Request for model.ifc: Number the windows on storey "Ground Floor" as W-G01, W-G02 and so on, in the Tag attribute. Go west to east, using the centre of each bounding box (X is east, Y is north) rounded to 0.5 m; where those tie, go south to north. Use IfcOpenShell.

First a look at what the model holds.

```python
import ifcopenshell
import ifcopenshell.util.element
import ifcopenshell.util.placement

model = ifcopenshell.open("model.ifc")
print(model.schema)
storey = next(s for s in model.by_type("IfcBuildingStorey") if s.Name == "Ground Floor")
windows = [e for e in ifcopenshell.util.element.get_decomposition(storey) if e.is_a("IfcWindow")]
for e in sorted(windows, key=lambda e: e.id()):
    origin = ifcopenshell.util.placement.get_local_placement(e.ObjectPlacement)[:3, 3]
    print(e.id(), e.Tag, e.Name, origin.round(2) + 0.0, sep=" | ")
```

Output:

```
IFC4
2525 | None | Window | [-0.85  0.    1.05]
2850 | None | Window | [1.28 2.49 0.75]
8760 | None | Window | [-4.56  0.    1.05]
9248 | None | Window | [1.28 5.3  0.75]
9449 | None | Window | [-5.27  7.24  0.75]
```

```python
import ifcopenshell
import ifcopenshell.geom
import ifcopenshell.util.element
import ifcopenshell.util.shape

model = ifcopenshell.open("model.ifc")
settings = ifcopenshell.geom.settings()
settings.set("use-world-coords", True)


def centre(element):
    shape = ifcopenshell.geom.create_shape(settings, element)
    return ifcopenshell.util.shape.get_bbox_centroid(shape.geometry)


storey = next(s for s in model.by_type("IfcBuildingStorey") if s.Name == "Ground Floor")
windows = [e for e in ifcopenshell.util.element.get_decomposition(storey) if e.is_a("IfcWindow")]

# Insertion points can sit at a corner or the storey origin, so sort by the geometry (in metres).
centres = {e: centre(e) for e in windows}
windows.sort(key=lambda e: (round(centres[e][0] / 0.5), centres[e][1]))

for i, e in enumerate(windows, start=1):
    number = f"W-G{i:02d}"
    e.Tag = number
    print(e.id(), number)

model.write("model_v2.ifc")
```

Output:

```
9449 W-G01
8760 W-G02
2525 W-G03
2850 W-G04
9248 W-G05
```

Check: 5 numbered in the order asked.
